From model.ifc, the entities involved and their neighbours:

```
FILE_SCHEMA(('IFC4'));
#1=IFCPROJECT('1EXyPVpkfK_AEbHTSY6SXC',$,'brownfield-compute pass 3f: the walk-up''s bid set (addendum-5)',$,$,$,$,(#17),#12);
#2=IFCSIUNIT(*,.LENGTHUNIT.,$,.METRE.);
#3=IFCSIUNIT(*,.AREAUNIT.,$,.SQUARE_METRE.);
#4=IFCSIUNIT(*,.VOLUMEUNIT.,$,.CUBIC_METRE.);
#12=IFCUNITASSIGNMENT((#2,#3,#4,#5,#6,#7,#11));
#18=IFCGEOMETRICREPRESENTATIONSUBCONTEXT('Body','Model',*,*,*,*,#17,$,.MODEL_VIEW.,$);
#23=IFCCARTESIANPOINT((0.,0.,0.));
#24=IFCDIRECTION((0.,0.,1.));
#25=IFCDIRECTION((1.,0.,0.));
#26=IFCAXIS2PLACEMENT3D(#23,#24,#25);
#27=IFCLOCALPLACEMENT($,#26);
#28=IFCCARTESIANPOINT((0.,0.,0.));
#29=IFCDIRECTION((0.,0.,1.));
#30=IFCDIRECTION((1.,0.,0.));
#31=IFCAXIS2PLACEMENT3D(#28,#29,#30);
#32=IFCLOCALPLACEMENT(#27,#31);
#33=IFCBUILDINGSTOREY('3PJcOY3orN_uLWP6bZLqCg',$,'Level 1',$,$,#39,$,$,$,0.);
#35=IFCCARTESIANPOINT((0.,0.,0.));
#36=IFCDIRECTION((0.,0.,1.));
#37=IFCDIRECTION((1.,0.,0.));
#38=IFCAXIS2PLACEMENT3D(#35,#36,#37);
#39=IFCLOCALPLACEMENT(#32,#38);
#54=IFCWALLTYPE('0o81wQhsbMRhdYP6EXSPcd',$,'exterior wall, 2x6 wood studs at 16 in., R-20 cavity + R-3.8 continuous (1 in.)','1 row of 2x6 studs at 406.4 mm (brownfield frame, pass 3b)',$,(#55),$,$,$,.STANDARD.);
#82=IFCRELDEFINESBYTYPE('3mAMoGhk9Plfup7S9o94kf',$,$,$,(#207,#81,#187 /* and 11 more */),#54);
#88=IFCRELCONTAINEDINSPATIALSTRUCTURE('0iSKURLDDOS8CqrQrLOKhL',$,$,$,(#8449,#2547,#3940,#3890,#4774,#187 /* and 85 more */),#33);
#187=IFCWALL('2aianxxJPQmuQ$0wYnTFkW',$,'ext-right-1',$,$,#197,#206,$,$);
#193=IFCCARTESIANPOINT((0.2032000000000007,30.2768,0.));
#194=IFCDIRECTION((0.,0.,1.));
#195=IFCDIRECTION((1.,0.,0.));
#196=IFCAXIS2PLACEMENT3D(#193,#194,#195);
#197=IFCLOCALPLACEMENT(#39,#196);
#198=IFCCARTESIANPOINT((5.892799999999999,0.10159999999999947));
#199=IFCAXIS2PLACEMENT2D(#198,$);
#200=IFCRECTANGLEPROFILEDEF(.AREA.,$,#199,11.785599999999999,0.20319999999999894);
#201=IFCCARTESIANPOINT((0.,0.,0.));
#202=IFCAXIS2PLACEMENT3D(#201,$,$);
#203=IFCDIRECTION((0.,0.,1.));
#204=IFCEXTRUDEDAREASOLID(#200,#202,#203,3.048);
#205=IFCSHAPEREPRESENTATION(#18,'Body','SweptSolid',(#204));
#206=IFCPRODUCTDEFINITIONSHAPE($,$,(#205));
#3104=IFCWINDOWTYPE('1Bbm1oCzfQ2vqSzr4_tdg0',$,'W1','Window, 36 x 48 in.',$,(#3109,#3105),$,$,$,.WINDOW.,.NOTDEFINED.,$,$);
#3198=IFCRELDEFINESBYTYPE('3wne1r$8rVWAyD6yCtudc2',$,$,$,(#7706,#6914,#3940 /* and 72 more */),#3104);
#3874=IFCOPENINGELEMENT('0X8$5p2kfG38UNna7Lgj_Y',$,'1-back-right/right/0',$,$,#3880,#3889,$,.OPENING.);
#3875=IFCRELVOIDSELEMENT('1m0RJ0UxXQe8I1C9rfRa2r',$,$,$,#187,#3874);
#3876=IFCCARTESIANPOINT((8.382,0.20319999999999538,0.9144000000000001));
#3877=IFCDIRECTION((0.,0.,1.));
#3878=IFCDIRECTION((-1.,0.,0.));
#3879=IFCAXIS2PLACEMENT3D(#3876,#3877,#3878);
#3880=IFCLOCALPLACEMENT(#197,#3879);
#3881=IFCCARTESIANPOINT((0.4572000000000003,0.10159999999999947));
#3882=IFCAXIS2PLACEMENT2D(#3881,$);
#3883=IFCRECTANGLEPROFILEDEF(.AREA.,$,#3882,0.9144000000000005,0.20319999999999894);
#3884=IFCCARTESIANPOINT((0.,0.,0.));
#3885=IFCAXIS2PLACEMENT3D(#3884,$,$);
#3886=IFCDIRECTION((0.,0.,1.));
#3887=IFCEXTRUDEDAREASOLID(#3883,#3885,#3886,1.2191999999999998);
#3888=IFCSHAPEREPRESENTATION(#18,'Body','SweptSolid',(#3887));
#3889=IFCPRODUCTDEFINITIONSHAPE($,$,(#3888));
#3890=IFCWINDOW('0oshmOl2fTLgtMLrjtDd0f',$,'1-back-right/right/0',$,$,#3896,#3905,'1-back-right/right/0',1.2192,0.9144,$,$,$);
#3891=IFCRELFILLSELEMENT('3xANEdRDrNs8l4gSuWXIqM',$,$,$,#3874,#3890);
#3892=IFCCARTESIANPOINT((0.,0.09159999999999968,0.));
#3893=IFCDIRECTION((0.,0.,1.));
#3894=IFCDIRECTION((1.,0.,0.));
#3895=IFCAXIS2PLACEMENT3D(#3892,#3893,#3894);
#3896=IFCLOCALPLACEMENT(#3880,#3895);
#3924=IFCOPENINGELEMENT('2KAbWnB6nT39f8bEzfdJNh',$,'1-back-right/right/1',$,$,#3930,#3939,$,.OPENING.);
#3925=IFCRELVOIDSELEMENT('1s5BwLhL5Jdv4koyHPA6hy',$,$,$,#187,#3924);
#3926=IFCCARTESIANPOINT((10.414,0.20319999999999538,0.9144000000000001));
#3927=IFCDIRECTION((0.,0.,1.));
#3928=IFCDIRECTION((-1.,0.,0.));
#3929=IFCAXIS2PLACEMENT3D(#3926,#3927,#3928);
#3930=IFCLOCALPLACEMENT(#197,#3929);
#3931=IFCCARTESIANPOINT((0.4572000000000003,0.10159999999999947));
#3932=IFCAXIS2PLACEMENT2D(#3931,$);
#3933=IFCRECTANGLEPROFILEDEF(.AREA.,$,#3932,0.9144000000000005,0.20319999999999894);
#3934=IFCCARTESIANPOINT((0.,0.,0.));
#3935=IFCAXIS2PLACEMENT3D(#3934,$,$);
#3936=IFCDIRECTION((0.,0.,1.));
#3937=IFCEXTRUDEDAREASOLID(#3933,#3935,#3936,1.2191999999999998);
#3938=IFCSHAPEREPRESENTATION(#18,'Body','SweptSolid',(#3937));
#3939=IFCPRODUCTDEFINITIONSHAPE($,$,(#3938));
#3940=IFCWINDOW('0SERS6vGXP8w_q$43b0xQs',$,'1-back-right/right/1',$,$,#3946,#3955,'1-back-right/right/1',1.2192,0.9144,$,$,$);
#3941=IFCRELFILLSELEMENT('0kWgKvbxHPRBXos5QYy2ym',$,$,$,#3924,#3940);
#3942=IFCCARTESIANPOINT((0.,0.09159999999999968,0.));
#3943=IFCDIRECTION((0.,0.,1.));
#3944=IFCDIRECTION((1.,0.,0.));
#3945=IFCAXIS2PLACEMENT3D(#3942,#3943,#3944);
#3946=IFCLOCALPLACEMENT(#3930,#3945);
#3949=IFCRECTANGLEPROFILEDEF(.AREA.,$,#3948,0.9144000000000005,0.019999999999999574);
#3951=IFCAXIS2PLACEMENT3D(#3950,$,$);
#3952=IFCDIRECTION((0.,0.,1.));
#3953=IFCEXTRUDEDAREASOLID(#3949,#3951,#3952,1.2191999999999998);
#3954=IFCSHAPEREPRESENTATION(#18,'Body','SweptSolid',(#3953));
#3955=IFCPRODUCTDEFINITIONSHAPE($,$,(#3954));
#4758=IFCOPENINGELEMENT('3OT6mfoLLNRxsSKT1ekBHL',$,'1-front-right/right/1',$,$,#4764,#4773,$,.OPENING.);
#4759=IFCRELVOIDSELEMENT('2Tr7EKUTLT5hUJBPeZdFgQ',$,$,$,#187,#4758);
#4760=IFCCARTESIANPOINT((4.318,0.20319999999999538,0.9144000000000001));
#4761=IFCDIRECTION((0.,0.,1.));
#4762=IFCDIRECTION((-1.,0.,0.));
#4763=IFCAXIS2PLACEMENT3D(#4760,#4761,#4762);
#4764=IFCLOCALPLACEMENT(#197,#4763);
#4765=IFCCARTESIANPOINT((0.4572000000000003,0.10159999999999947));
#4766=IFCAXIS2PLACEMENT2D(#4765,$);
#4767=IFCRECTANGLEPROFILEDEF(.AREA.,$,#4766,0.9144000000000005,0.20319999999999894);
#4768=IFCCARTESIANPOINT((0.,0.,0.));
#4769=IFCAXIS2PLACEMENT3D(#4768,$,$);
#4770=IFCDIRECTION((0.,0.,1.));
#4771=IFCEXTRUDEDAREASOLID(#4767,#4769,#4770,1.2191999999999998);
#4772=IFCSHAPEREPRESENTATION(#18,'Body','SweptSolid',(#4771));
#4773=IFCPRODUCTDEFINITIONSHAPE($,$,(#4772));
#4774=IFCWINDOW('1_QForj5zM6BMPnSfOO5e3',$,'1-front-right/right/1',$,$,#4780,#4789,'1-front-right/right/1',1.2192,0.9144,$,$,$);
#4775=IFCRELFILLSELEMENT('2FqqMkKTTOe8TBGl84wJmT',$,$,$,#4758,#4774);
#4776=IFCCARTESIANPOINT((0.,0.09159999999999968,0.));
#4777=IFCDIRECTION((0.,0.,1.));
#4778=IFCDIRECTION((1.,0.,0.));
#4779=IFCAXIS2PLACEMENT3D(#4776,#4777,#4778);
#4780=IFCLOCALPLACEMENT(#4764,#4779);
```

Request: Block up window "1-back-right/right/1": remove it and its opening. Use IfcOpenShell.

```python
import ifcopenshell
import ifcopenshell.api.feature
import ifcopenshell.api.root
import ifcopenshell.geom
import ifcopenshell.util.shape

model = ifcopenshell.open("model.ifc")
settings = ifcopenshell.geom.settings()


def volume(element):
    """Net volume in cubic metres, openings subtracted."""
    shape = ifcopenshell.geom.create_shape(settings, element)
    return ifcopenshell.util.shape.get_volume(shape.geometry)


window = model.by_guid("0SERS6vGXP8w_q$43b0xQs")
opening = window.FillsVoids[0].RelatingOpeningElement
wall = opening.VoidsElements[0].RelatingBuildingElement
before = volume(wall)

ifcopenshell.api.root.remove_product(model, product=window)
ifcopenshell.api.feature.remove_feature(model, feature=opening)

after = volume(wall)

print(f"wall volume {before:.3f} -> {after:.3f} m3")

model.write("model_updated.ifc")
```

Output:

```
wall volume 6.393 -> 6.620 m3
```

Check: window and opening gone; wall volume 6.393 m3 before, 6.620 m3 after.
